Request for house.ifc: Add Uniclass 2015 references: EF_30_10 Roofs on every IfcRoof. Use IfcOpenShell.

First a look at what the model holds.

```python
import ifcopenshell

model = ifcopenshell.open("house.ifc")
print(model.schema)
print("classifications:", [c.Name for c in model.by_type("IfcClassification")])
for ifc_class in ("IfcDoor", "IfcRoof", "IfcStair", "IfcWall", "IfcWindow"):
    print(ifc_class, len(model.by_type(ifc_class)))
```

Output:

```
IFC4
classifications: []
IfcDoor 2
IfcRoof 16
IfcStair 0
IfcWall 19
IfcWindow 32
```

```python
import ifcopenshell
import ifcopenshell.api.classification

model = ifcopenshell.open("house.ifc")

system = ifcopenshell.api.classification.add_classification(model, classification="Uniclass 2015")

codes = {
    "IfcRoof": ("EF_30_10", "Roofs"),
}
for ifc_class, (code, name) in codes.items():
    products = model.by_type(ifc_class)
    ifcopenshell.api.classification.add_reference(
        model, products=products, classification=system, identification=code, name=name
    )
    print(code, len(products))

model.write("house_rev.ifc")
```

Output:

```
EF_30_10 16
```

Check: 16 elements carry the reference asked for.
